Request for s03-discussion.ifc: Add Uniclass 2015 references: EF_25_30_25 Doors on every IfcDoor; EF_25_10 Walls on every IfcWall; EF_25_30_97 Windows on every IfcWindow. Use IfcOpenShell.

First a look at what the model holds.

```python
import ifcopenshell

model = ifcopenshell.open("s03-discussion.ifc")
print(model.schema)
print("classifications:", [c.Name for c in model.by_type("IfcClassification")])
for ifc_class in ("IfcDoor", "IfcRoof", "IfcStair", "IfcWall", "IfcWindow"):
    print(ifc_class, len(model.by_type(ifc_class)))
```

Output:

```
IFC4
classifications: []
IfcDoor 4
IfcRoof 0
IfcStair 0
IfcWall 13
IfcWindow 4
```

```python
import ifcopenshell
import ifcopenshell.api.classification

model = ifcopenshell.open("s03-discussion.ifc")

system = ifcopenshell.api.classification.add_classification(model, classification="Uniclass 2015")

codes = {
    "IfcDoor": ("EF_25_30_25", "Doors"),
    "IfcWall": ("EF_25_10", "Walls"),
    "IfcWindow": ("EF_25_30_97", "Windows"),
}
for ifc_class, (code, name) in codes.items():
    products = model.by_type(ifc_class)
    ifcopenshell.api.classification.add_reference(
        model, products=products, classification=system, identification=code, name=name
    )
    print(code, len(products))

model.write("s03-discussion_edited.ifc")
```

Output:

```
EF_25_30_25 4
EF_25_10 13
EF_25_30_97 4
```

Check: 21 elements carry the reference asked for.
